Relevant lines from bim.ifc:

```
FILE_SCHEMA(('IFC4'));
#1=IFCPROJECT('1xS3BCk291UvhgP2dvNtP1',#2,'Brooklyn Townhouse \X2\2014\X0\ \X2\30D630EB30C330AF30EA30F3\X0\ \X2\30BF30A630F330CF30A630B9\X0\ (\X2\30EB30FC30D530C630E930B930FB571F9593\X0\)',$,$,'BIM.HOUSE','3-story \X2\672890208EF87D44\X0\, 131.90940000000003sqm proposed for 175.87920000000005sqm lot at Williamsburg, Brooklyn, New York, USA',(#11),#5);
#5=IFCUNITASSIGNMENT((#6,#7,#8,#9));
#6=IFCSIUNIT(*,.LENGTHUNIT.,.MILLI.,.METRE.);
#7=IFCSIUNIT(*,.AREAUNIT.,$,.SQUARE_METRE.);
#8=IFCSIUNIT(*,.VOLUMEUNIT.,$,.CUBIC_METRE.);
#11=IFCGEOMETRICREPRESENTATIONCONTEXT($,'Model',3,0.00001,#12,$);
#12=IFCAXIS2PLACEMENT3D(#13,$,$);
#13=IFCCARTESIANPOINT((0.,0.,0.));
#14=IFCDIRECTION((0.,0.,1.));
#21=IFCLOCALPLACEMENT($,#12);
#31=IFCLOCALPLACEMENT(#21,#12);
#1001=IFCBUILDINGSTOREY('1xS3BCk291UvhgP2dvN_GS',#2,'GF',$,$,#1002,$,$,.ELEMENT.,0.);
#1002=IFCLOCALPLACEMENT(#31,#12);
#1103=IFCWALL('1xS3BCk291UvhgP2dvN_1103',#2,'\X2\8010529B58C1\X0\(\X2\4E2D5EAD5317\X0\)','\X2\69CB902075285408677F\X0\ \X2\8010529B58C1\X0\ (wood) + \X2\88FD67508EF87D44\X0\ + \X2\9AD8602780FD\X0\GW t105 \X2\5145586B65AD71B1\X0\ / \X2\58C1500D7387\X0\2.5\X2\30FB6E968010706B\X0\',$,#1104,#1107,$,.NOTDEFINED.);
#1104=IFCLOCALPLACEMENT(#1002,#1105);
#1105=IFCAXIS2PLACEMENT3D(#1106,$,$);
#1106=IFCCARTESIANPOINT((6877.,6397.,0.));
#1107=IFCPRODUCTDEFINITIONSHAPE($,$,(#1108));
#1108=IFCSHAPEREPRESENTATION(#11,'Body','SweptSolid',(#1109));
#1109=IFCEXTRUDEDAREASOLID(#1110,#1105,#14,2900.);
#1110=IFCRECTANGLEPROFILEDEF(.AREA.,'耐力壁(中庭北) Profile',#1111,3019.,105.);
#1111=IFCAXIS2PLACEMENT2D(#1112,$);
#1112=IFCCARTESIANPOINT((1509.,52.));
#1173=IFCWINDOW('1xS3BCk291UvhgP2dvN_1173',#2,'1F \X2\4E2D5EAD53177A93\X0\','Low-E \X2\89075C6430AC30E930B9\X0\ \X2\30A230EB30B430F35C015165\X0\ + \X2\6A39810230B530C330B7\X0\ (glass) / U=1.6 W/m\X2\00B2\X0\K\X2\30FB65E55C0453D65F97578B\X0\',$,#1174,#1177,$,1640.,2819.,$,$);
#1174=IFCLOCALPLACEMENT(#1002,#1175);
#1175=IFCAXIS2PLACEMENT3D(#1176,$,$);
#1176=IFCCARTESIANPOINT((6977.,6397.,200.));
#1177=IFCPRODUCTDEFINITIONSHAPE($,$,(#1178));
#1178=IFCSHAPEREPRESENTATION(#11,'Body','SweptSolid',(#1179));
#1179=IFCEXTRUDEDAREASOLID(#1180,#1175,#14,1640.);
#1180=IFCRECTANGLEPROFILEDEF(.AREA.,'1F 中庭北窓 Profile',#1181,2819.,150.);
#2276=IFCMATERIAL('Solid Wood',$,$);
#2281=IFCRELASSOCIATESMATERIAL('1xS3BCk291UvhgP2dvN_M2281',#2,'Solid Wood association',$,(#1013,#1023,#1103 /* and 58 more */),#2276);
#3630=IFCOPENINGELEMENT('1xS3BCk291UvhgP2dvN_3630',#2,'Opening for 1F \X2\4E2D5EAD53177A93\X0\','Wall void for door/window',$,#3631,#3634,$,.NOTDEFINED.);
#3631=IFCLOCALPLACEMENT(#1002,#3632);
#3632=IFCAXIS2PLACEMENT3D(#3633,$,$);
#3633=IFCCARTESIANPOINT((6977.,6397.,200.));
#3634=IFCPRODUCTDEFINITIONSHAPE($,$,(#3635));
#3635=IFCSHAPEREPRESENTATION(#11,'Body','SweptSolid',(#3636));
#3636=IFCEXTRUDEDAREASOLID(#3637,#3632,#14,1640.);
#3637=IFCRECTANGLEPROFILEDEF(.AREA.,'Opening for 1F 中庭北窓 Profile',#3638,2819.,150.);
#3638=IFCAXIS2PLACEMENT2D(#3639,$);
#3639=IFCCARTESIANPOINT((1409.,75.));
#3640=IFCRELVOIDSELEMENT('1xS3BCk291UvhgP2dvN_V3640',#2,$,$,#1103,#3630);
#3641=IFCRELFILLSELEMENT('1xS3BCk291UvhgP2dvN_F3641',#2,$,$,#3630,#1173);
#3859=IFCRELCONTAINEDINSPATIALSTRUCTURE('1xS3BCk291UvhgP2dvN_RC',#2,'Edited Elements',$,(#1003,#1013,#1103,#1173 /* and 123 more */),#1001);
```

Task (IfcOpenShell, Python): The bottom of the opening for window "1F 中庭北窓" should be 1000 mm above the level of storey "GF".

```python
import numpy as np
import ifcopenshell
import ifcopenshell.api.geometry
import ifcopenshell.geom
import ifcopenshell.util.element
import ifcopenshell.util.placement
import ifcopenshell.util.shape
import ifcopenshell.util.unit

model = ifcopenshell.open("bim.ifc")
unit_scale = ifcopenshell.util.unit.calculate_unit_scale(model)

window = model.by_id(1173)
opening = window.FillsVoids[0].RelatingOpeningElement
storey = ifcopenshell.util.element.get_container(window, ifc_class="IfcBuildingStorey")
level = ifcopenshell.util.placement.get_local_placement(storey.ObjectPlacement)[2, 3]

# The opening's origin need not be at the sill, so measure its lowest point.
shape = ifcopenshell.geom.create_shape(ifcopenshell.geom.settings(), opening)
bottom = ifcopenshell.util.shape.get_shape_bottom_elevation(shape, shape.geometry) / unit_scale
dz = level + 1 / unit_scale - bottom

shift = np.array([0.0, 0.0, dz])
# The window is not placed relative to its opening, so move both.
for product in (opening, window):
    matrix = ifcopenshell.util.placement.get_local_placement(product.ObjectPlacement)
    matrix[:3, 3] += shift
    ifcopenshell.api.geometry.edit_object_placement(model, product=product, matrix=matrix, is_si=False)

print(f"moved by {dz * unit_scale:+.3f} m")

model.write("bim_v2.ifc")
```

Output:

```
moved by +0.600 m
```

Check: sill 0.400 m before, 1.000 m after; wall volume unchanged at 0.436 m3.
